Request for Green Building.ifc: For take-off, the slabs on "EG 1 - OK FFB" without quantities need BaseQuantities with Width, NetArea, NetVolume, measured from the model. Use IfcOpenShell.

First a look at what the model holds.

```python
import ifcopenshell
import ifcopenshell.util.element
import ifcopenshell.util.unit

model = ifcopenshell.open("Green Building.ifc")
print(model.schema)
for unit_type in ("LENGTHUNIT", "AREAUNIT", "VOLUMEUNIT"):
    print(unit_type, ifcopenshell.util.unit.calculate_unit_scale(model, unit_type))
storey = next(s for s in model.by_type("IfcBuildingStorey") if s.Name == "EG 1 - OK FFB")
slabs = [e for e in ifcopenshell.util.element.get_decomposition(storey) if e.is_a("IfcSlab")]
for e in sorted(slabs, key=lambda e: e.id()):
    print(e.id(), e.is_a(), e.Name, list(ifcopenshell.util.element.get_psets(e, qtos_only=True)), sep=" | ")
```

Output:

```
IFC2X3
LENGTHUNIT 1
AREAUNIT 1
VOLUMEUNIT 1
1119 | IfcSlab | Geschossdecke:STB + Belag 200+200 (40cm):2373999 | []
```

```python
import ifcopenshell
import ifcopenshell.api.pset
import ifcopenshell.geom
import ifcopenshell.util.element
import ifcopenshell.util.shape
import ifcopenshell.util.unit

model = ifcopenshell.open("Green Building.ifc")
unit_scale = ifcopenshell.util.unit.calculate_unit_scale(model)
area_scale = ifcopenshell.util.unit.calculate_unit_scale(model, "AREAUNIT")
volume_scale = ifcopenshell.util.unit.calculate_unit_scale(model, "VOLUMEUNIT")
settings = ifcopenshell.geom.settings()

storey = next(s for s in model.by_type("IfcBuildingStorey") if s.Name == "EG 1 - OK FFB")
slabs = [e for e in ifcopenshell.util.element.get_decomposition(storey) if e.is_a("IfcSlab")]

for e in sorted(slabs, key=lambda e: e.id()):
    if ifcopenshell.util.element.get_psets(e, qtos_only=True, should_inherit=False):
        continue
    # Geometry comes back in metres, in the element's own axes.
    shape = ifcopenshell.geom.create_shape(settings, e)
    values = {
        "Width": ifcopenshell.util.shape.get_z(shape.geometry) / unit_scale,
        "NetArea": ifcopenshell.util.shape.get_footprint_area(shape.geometry) / area_scale,
        "NetVolume": ifcopenshell.util.shape.get_volume(shape.geometry) / volume_scale,
    }
    qto = ifcopenshell.api.pset.add_qto(model, product=e, name="BaseQuantities")
    ifcopenshell.api.pset.edit_qto(model, qto=qto, properties=values)
    print(e.id(), {k: round(v, 3) for k, v in values.items()})

model.write("Green Building_edited.ifc")
```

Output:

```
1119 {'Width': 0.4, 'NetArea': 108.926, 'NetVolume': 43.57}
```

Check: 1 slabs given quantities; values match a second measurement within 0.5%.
